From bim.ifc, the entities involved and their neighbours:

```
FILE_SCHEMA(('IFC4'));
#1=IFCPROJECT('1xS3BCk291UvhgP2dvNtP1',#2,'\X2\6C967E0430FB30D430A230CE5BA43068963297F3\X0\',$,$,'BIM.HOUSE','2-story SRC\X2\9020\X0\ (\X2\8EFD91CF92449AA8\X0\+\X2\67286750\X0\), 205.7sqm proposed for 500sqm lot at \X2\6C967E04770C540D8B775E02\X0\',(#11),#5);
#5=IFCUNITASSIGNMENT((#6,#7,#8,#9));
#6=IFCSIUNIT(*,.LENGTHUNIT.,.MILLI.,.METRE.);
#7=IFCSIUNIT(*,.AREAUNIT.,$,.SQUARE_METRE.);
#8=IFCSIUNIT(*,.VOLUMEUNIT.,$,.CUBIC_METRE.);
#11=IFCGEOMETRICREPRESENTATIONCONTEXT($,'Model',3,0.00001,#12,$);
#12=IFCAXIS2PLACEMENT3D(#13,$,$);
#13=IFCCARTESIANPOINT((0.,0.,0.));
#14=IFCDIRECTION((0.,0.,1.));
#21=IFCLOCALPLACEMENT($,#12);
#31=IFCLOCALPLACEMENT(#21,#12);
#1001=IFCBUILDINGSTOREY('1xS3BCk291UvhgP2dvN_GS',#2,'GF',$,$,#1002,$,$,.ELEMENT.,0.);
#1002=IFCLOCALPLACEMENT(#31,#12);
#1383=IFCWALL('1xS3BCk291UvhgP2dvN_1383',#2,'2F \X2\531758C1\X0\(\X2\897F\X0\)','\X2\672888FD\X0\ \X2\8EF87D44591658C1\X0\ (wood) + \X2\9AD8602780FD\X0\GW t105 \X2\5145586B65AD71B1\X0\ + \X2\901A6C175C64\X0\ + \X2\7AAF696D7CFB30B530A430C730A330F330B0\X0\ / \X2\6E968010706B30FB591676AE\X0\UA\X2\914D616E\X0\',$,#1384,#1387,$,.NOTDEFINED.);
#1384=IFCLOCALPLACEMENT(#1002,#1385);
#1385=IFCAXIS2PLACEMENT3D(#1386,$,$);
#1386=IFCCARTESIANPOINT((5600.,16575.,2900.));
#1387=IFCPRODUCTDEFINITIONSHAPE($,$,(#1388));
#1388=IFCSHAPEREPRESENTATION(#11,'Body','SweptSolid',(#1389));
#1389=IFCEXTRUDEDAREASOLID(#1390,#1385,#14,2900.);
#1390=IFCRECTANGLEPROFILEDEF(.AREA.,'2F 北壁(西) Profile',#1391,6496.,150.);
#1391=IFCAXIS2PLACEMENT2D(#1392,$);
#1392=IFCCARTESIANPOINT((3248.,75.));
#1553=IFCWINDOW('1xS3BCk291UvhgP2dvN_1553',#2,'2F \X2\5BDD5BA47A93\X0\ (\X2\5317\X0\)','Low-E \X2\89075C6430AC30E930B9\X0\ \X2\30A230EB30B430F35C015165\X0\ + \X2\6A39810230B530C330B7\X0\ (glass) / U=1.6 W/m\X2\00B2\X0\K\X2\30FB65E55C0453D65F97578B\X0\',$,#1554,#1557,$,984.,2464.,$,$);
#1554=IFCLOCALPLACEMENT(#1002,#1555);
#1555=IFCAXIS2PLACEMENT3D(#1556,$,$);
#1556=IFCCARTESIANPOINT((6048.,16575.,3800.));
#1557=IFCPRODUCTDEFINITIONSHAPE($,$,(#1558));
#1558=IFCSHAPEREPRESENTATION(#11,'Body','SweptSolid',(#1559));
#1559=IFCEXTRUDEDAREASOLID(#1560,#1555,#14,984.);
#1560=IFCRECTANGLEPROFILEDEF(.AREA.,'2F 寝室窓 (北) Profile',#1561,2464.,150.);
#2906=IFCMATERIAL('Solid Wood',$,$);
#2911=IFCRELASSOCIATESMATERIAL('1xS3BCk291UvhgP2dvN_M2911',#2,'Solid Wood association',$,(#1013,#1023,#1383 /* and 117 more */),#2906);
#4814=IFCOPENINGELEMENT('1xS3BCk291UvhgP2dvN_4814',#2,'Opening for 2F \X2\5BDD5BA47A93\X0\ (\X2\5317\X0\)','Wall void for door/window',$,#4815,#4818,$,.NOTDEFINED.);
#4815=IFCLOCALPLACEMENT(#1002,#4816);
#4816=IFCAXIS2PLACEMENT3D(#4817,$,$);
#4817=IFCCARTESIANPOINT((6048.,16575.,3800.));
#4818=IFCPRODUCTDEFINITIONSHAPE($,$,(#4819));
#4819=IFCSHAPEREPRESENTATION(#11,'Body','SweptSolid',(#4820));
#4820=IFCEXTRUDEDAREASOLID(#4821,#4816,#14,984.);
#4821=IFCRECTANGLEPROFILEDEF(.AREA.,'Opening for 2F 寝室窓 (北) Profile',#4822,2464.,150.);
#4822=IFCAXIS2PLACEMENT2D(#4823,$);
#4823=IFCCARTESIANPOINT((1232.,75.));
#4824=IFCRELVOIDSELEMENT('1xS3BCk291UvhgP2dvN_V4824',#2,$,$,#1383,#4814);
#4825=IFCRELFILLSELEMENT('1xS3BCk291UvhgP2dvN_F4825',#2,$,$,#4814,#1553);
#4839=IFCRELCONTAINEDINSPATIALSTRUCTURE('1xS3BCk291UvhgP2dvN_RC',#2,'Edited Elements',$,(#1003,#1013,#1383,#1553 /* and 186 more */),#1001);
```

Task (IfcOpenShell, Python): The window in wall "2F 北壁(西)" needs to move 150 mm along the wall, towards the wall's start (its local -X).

```python
import ifcopenshell
import ifcopenshell.api.geometry
import ifcopenshell.util.placement
import ifcopenshell.util.unit

model = ifcopenshell.open("bim.ifc")
unit_scale = ifcopenshell.util.unit.calculate_unit_scale(model)

window = model.by_guid("1xS3BCk291UvhgP2dvN_1553")
opening = window.FillsVoids[0].RelatingOpeningElement
wall = opening.VoidsElements[0].RelatingBuildingElement

wall_matrix = ifcopenshell.util.placement.get_local_placement(wall.ObjectPlacement)
shift = wall_matrix[:3, 0] * -0.15 / unit_scale
before = ifcopenshell.util.placement.get_local_placement(window.ObjectPlacement)[:3, 3].copy()

# The window is not placed relative to its opening, so move both.
for product in (opening, window):
    matrix = ifcopenshell.util.placement.get_local_placement(product.ObjectPlacement)
    matrix[:3, 3] += shift
    ifcopenshell.api.geometry.edit_object_placement(model, product=product, matrix=matrix, is_si=False)

after = ifcopenshell.util.placement.get_local_placement(window.ObjectPlacement)[:3, 3]
print("window moved by", (after - before).round(3) + 0.0)

model.write("bim_v2.ifc")
```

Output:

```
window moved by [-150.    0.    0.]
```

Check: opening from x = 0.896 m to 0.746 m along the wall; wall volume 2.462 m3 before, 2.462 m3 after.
